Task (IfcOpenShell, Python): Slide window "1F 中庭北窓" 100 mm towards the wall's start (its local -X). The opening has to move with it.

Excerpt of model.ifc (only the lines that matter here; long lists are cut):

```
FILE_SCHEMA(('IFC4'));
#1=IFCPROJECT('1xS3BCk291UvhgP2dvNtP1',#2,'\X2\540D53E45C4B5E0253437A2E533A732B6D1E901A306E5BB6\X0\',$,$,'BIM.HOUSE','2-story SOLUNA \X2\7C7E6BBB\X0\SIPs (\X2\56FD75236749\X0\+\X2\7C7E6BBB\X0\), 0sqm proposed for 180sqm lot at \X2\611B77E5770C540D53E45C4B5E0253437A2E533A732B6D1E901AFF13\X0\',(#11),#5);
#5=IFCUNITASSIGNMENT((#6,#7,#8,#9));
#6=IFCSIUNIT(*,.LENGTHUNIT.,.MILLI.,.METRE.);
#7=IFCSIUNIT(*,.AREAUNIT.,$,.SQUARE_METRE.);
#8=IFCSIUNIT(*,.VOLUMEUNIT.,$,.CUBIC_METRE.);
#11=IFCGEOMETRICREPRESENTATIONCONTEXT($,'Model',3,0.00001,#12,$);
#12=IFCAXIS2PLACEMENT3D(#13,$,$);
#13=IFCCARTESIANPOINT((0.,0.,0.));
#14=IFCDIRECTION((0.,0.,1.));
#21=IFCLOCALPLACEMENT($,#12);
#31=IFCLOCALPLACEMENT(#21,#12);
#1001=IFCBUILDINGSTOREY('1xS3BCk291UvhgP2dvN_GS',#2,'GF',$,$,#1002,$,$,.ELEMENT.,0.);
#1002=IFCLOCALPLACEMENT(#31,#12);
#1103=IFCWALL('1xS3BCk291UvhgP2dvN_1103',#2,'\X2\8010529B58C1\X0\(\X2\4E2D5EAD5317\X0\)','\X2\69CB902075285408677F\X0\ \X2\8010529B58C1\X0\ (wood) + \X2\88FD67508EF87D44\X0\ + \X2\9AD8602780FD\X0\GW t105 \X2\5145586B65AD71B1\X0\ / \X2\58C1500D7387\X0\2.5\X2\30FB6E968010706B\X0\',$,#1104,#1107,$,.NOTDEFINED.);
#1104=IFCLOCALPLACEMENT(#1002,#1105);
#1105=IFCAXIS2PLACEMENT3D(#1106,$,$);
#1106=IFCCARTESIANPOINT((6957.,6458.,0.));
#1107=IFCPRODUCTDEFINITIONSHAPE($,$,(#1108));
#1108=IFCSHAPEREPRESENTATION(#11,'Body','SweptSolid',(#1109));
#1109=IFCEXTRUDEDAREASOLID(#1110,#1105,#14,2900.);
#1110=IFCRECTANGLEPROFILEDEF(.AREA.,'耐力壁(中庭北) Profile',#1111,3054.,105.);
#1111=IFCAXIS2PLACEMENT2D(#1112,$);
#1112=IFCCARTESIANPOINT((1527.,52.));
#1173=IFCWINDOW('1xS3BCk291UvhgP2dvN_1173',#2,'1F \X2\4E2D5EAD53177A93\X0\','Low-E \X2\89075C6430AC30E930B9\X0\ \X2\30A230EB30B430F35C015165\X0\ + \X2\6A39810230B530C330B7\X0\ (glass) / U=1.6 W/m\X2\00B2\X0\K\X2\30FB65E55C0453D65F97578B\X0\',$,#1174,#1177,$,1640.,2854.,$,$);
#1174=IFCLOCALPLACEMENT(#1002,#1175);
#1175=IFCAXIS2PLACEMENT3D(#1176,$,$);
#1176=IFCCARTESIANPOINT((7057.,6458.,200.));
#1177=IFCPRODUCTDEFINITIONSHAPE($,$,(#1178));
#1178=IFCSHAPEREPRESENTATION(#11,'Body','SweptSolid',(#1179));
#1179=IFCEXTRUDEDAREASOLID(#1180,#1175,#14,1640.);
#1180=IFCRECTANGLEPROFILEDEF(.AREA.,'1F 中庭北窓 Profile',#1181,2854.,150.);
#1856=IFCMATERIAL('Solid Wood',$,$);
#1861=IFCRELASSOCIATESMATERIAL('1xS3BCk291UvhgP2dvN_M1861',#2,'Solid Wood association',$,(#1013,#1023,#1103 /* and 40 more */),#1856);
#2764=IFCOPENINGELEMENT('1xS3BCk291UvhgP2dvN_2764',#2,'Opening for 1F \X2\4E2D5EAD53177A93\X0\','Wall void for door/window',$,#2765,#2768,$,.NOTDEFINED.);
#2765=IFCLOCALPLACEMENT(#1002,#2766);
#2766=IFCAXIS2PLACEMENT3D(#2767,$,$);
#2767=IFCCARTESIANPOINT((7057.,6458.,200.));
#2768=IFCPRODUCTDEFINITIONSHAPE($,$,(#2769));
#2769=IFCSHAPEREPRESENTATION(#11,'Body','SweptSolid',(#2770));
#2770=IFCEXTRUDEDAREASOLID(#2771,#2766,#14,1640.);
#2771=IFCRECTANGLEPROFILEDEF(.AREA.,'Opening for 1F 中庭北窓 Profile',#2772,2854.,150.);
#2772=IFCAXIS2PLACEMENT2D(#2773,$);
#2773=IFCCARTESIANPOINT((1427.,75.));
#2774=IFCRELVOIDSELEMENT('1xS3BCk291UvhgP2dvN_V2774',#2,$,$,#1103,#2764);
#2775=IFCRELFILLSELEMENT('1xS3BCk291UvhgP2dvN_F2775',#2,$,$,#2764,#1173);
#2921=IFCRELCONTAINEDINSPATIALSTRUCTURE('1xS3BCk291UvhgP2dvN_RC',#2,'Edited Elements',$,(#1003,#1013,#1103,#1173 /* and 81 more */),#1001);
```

```python
import ifcopenshell
import ifcopenshell.api.geometry
import ifcopenshell.util.placement
import ifcopenshell.util.unit

model = ifcopenshell.open("model.ifc")
unit_scale = ifcopenshell.util.unit.calculate_unit_scale(model)

window = model.by_guid("1xS3BCk291UvhgP2dvN_1173")
opening = window.FillsVoids[0].RelatingOpeningElement
wall = opening.VoidsElements[0].RelatingBuildingElement

wall_matrix = ifcopenshell.util.placement.get_local_placement(wall.ObjectPlacement)
shift = wall_matrix[:3, 0] * -0.1 / unit_scale
before = ifcopenshell.util.placement.get_local_placement(window.ObjectPlacement)[:3, 3].copy()

# The window is not placed relative to its opening, so move both.
for product in (opening, window):
    matrix = ifcopenshell.util.placement.get_local_placement(product.ObjectPlacement)
    matrix[:3, 3] += shift
    ifcopenshell.api.geometry.edit_object_placement(model, product=product, matrix=matrix, is_si=False)

after = ifcopenshell.util.placement.get_local_placement(window.ObjectPlacement)[:3, 3]
print("window moved by", (after - before).round(3) + 0.0)

model.write("model_edited.ifc")
```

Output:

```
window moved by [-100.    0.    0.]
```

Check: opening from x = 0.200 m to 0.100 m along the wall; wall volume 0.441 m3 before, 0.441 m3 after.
